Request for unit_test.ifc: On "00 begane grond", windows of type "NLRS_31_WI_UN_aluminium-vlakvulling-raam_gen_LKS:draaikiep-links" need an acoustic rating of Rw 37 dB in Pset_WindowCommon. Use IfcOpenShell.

First a look at what the model holds.

```python
import ifcopenshell
import ifcopenshell.util.element

model = ifcopenshell.open("unit_test.ifc")
print(model.schema)
storey = next(s for s in model.by_type("IfcBuildingStorey") if s.Name == "00 begane grond")
windows = [e for e in ifcopenshell.util.element.get_decomposition(storey) if e.is_a("IfcWindow")]
seen = {}
for e in windows:
    element_type = ifcopenshell.util.element.get_type(e)
    key = (element_type.Name if element_type != e and element_type else None, ifcopenshell.util.element.get_pset(e, "Pset_WindowCommon", "AcousticRating"))
    seen[key] = seen.get(key, 0) + 1
for (name, value), count in sorted(seen.items(), key=str):
    print(count, "x", name, "|", value)
```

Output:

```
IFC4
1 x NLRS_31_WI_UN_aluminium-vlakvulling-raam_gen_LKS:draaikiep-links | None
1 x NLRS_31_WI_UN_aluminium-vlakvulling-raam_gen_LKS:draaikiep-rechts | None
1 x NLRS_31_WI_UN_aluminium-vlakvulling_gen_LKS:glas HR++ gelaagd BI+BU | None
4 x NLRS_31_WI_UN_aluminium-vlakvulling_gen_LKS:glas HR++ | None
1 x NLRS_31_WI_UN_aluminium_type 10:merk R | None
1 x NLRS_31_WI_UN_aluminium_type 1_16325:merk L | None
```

```python
import ifcopenshell
import ifcopenshell.api.pset
import ifcopenshell.util.element

model = ifcopenshell.open("unit_test.ifc")

storey = next(s for s in model.by_type("IfcBuildingStorey") if s.Name == "00 begane grond")
windows = [e for e in ifcopenshell.util.element.get_decomposition(storey) if e.is_a("IfcWindow")]

count = 0
for e in windows:
    element_type = ifcopenshell.util.element.get_type(e)
    if element_type in (None, e) or element_type.Name != "NLRS_31_WI_UN_aluminium-vlakvulling-raam_gen_LKS:draaikiep-links":
        continue
    # add_pset returns the element's existing set when there is one.
    pset = ifcopenshell.api.pset.add_pset(model, product=e, name="Pset_WindowCommon")
    ifcopenshell.api.pset.edit_pset(model, pset=pset, properties={"AcousticRating": "Rw 37 dB"})
    count += 1

print(count, "windows updated")

model.write("unit_test_rev.ifc")
```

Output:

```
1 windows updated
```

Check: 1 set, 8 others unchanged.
